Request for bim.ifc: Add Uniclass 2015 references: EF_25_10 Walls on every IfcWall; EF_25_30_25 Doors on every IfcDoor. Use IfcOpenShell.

First a look at what the model holds.

```python
import ifcopenshell

model = ifcopenshell.open("bim.ifc")
print(model.schema)
print("classifications:", [c.Name for c in model.by_type("IfcClassification")])
for ifc_class in ("IfcDoor", "IfcRoof", "IfcStair", "IfcWall", "IfcWindow"):
    print(ifc_class, len(model.by_type(ifc_class)))
```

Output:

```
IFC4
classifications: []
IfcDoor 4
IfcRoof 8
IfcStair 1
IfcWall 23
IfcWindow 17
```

```python
import ifcopenshell
import ifcopenshell.api.classification

model = ifcopenshell.open("bim.ifc")

system = ifcopenshell.api.classification.add_classification(model, classification="Uniclass 2015")

codes = {
    "IfcWall": ("EF_25_10", "Walls"),
    "IfcDoor": ("EF_25_30_25", "Doors"),
}
for ifc_class, (code, name) in codes.items():
    products = model.by_type(ifc_class)
    ifcopenshell.api.classification.add_reference(
        model, products=products, classification=system, identification=code, name=name
    )
    print(code, len(products))

model.write("bim_rev.ifc")
```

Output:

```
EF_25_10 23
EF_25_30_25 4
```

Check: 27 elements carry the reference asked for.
